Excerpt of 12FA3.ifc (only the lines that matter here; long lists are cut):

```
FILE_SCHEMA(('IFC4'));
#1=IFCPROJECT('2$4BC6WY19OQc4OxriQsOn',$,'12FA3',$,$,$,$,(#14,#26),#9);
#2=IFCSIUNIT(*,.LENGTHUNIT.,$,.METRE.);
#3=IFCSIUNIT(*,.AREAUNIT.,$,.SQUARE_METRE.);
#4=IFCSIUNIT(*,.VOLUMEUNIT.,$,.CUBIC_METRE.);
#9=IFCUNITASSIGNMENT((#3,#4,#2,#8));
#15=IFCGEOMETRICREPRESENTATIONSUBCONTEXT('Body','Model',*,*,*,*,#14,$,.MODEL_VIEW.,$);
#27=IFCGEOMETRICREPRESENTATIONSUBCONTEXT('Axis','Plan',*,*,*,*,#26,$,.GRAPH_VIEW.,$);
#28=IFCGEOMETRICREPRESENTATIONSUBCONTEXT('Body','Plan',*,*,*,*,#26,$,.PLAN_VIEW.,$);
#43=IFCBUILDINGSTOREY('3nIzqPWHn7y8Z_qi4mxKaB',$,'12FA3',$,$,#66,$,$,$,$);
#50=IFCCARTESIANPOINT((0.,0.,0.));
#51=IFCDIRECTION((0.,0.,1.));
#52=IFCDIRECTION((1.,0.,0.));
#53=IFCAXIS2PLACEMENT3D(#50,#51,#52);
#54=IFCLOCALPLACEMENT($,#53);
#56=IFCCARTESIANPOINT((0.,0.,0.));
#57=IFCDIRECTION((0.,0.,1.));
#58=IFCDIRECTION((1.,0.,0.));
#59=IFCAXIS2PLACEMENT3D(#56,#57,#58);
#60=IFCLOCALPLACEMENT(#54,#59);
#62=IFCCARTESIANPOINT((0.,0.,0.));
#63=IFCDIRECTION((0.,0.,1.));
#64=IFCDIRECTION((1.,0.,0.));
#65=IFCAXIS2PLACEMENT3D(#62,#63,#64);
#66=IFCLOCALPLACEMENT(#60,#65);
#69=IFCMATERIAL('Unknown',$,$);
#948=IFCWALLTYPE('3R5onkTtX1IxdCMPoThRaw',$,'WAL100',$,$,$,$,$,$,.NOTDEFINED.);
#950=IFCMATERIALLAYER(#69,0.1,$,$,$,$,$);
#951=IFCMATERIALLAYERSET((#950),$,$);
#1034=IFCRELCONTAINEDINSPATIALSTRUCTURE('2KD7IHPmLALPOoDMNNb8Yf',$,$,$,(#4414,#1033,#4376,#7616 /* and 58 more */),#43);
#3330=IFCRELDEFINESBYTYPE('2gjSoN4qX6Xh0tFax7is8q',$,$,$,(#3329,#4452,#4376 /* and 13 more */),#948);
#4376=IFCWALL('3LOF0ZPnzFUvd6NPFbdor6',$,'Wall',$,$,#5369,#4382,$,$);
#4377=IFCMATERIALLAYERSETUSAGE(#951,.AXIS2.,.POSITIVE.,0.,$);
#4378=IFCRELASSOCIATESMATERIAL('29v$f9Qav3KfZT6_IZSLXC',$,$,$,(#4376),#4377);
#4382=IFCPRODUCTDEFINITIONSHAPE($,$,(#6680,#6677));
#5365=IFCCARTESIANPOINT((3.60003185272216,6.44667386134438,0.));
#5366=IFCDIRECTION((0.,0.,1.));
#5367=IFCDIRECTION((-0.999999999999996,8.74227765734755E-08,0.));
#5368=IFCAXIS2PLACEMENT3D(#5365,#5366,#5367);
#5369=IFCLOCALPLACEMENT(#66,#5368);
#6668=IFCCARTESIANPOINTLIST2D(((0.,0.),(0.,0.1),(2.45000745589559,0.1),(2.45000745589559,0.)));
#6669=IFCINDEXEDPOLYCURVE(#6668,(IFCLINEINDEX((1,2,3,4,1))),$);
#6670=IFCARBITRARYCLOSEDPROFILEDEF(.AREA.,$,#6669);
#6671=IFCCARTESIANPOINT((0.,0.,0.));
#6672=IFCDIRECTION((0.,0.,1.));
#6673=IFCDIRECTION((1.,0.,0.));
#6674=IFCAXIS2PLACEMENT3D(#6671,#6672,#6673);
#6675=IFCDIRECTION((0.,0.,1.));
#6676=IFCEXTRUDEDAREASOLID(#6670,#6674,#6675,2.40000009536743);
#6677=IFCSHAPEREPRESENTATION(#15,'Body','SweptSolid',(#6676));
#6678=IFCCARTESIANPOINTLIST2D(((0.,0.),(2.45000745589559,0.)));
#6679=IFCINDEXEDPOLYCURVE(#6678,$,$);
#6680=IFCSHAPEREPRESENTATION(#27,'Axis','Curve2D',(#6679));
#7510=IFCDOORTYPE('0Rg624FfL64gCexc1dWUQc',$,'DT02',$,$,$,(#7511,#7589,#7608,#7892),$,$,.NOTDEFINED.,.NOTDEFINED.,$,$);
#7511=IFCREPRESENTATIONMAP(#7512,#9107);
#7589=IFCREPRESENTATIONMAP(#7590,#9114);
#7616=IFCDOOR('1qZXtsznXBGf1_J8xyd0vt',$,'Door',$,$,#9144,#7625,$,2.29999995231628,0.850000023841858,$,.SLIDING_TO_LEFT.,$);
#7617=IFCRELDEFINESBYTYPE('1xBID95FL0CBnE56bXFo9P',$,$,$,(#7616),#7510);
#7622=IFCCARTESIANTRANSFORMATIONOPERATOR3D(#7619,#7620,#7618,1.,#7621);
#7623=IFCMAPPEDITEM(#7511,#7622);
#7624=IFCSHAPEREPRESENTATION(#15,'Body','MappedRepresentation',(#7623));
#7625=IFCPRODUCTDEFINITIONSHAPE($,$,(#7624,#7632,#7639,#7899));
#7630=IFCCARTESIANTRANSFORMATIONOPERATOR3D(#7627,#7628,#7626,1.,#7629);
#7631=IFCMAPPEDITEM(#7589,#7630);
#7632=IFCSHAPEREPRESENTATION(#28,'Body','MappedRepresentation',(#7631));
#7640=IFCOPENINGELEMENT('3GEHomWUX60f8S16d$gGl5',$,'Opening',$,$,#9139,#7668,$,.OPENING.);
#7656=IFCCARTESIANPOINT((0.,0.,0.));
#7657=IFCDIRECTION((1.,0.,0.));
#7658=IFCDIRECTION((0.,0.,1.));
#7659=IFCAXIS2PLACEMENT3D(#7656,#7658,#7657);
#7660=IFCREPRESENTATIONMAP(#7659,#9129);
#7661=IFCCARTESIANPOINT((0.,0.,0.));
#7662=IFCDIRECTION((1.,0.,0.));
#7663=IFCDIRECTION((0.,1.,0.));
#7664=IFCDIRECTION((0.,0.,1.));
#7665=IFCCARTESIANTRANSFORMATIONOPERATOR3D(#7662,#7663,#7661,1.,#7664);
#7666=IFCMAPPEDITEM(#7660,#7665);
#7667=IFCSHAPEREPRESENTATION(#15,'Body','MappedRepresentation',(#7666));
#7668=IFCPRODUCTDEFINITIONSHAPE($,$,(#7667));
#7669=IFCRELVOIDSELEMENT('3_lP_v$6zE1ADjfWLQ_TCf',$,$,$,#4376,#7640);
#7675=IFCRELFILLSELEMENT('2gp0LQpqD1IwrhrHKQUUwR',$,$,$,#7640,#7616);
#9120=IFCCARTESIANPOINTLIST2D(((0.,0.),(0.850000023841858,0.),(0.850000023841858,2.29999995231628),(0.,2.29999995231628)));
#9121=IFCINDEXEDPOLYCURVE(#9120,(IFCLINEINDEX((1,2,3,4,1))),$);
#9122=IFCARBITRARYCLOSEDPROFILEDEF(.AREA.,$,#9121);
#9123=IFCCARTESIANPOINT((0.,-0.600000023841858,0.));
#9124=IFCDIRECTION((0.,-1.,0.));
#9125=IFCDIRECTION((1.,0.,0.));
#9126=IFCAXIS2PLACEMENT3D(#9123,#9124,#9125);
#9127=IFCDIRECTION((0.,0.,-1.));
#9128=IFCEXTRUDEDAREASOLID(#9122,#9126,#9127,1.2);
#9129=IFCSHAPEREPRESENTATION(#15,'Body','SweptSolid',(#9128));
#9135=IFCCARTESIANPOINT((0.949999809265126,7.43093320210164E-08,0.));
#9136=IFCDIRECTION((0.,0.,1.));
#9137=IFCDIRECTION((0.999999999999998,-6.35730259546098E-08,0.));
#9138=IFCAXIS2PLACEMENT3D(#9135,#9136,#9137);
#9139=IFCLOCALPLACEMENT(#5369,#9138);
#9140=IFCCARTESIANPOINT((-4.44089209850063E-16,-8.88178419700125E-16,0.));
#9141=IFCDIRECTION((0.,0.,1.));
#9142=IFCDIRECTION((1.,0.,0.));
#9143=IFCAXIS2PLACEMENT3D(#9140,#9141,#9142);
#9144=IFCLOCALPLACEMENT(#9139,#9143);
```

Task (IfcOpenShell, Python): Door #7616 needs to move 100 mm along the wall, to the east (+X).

```python
import ifcopenshell
import ifcopenshell.api.geometry
import ifcopenshell.util.placement
import ifcopenshell.util.unit

model = ifcopenshell.open("12FA3.ifc")
unit_scale = ifcopenshell.util.unit.calculate_unit_scale(model)

door = model.by_guid("1qZXtsznXBGf1_J8xyd0vt")
opening = door.FillsVoids[0].RelatingOpeningElement
wall = opening.VoidsElements[0].RelatingBuildingElement

wall_matrix = ifcopenshell.util.placement.get_local_placement(wall.ObjectPlacement)
shift = wall_matrix[:3, 0] * -0.1 / unit_scale
before = ifcopenshell.util.placement.get_local_placement(door.ObjectPlacement)[:3, 3].copy()

# The door is placed relative to its opening, so it follows when the opening moves.
matrix = ifcopenshell.util.placement.get_local_placement(opening.ObjectPlacement)
matrix[:3, 3] += shift
ifcopenshell.api.geometry.edit_object_placement(
    model, product=opening, matrix=matrix, is_si=False, should_transform_children=True
)

after = ifcopenshell.util.placement.get_local_placement(door.ObjectPlacement)[:3, 3]
print("door moved by", (after - before).round(3) + 0.0)

model.write("12FA3-out.ifc")
```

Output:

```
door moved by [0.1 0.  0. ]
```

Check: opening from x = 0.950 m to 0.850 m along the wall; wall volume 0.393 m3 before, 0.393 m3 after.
